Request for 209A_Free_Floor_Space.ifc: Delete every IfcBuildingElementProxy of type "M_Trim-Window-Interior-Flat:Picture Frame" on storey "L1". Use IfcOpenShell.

First a look at what the model holds.

```python
import ifcopenshell
import ifcopenshell.util.element

model = ifcopenshell.open("209A_Free_Floor_Space.ifc")
print(model.schema)
storey = next(s for s in model.by_type("IfcBuildingStorey") if s.Name == "L1")
proxies = [e for e in ifcopenshell.util.element.get_decomposition(storey) if e.is_a("IfcBuildingElementProxy")]
seen = {}
for e in proxies:
    element_type = ifcopenshell.util.element.get_type(e)
    name = element_type.Name if element_type not in (None, e) else None
    seen[name] = seen.get(name, 0) + 1
for name, count in sorted(seen.items(), key=str):
    print(count, "x", name)
```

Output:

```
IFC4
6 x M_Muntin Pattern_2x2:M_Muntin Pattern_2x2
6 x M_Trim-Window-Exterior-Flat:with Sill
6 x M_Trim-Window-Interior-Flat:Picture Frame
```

```python
import ifcopenshell
import ifcopenshell.api.root
import ifcopenshell.util.element

model = ifcopenshell.open("209A_Free_Floor_Space.ifc")

storey = next(s for s in model.by_type("IfcBuildingStorey") if s.Name == "L1")
proxies = [e for e in ifcopenshell.util.element.get_decomposition(storey) if e.is_a("IfcBuildingElementProxy")]
targets = [e for e in proxies if (t := ifcopenshell.util.element.get_type(e)) not in (None, e) and t.Name == "M_Trim-Window-Interior-Flat:Picture Frame"]

for e in targets:
    ifcopenshell.api.root.remove_product(model, product=e)
print(len(targets), "removed")

model.write("209A_Free_Floor_Space_v2.ifc")
```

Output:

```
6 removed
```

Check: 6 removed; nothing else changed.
